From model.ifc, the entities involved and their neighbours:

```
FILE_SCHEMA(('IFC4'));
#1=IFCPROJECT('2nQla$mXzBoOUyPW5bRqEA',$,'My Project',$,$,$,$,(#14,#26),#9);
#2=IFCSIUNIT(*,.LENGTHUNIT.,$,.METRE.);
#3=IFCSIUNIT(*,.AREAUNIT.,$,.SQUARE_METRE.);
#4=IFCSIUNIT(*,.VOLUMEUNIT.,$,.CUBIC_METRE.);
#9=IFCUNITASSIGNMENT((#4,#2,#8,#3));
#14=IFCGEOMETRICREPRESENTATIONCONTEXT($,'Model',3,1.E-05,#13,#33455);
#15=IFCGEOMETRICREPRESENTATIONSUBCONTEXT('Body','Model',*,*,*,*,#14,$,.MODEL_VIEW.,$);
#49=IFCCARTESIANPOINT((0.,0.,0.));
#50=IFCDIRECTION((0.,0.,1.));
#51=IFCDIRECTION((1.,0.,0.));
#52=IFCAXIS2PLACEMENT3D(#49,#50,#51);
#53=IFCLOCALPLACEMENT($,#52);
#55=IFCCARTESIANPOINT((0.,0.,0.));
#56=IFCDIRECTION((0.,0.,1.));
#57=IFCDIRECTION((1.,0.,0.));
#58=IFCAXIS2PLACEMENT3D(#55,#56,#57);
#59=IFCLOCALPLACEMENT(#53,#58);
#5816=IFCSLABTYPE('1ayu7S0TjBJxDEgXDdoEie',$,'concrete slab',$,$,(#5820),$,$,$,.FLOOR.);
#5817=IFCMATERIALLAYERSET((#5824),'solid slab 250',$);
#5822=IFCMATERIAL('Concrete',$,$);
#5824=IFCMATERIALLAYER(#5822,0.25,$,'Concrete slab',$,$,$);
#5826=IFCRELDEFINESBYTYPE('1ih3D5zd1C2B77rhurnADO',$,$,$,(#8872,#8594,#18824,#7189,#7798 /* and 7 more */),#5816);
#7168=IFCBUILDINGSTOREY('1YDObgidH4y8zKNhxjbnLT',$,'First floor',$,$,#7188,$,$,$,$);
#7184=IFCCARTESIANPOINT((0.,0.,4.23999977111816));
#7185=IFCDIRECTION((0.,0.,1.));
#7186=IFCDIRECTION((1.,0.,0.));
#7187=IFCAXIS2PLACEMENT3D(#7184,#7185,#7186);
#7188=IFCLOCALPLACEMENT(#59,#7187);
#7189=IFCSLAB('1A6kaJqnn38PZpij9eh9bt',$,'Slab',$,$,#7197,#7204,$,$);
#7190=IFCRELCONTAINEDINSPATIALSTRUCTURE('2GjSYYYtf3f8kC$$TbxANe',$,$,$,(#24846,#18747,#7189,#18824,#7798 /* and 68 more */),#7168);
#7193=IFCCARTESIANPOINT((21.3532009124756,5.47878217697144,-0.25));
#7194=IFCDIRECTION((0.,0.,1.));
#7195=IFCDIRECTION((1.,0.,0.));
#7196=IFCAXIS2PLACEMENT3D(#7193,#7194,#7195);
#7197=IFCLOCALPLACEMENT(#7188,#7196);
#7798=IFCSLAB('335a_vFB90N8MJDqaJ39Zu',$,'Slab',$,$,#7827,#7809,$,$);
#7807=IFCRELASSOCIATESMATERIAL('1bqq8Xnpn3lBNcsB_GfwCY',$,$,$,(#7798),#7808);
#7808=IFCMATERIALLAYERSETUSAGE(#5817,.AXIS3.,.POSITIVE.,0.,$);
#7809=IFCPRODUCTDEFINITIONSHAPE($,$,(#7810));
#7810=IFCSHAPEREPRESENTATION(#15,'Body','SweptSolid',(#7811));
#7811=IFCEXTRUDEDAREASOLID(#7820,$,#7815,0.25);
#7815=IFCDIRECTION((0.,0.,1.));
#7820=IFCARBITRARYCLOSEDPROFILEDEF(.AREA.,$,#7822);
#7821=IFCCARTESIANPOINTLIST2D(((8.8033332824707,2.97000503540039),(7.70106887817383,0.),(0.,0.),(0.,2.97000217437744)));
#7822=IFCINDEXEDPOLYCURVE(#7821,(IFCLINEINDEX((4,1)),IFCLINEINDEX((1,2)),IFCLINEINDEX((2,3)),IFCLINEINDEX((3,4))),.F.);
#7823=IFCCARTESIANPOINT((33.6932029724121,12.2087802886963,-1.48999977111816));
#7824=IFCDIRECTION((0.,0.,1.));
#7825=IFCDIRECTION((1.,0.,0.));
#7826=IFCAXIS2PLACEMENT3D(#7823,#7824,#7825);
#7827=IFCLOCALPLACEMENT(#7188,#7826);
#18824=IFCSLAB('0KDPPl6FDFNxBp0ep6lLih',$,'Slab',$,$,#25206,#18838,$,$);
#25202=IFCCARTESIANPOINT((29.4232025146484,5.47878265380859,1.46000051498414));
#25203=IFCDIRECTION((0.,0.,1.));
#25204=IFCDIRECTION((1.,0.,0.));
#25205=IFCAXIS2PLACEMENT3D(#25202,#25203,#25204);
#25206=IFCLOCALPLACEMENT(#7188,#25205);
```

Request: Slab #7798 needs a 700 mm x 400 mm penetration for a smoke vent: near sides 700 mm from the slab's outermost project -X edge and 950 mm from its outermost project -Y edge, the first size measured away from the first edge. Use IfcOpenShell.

```python
import numpy as np
import ifcopenshell
import ifcopenshell.api.feature
import ifcopenshell.api.geometry
import ifcopenshell.api.root
import ifcopenshell.geom
import ifcopenshell.util.placement
import ifcopenshell.util.representation
import ifcopenshell.util.shape
import ifcopenshell.util.unit

model = ifcopenshell.open("model.ifc")
unit_scale = ifcopenshell.util.unit.calculate_unit_scale(model)
settings = ifcopenshell.geom.settings()


def volume(element):
    """Net volume in cubic metres, openings subtracted."""
    shape = ifcopenshell.geom.create_shape(settings, element)
    return ifcopenshell.util.shape.get_volume(shape.geometry)


slab = model.by_guid("335a_vFB90N8MJDqaJ39Zu")
before = volume(slab)

# Extent in the slab's own axes, in metres. The edges named are its -X and -Y sides.
slab_shape = ifcopenshell.geom.create_shape(settings, slab)
vertices = ifcopenshell.util.shape.get_vertices(slab_shape.geometry)
x_min, y_min, bottom = vertices.min(axis=0)
top = vertices[:, 2].max()

opening = ifcopenshell.api.root.create_entity(model, ifc_class="IfcOpeningElement", name="Smoke vent opening", predefined_type="OPENING")
context = ifcopenshell.util.representation.get_context(model, "Model", "Body", "MODEL_VIEW")
width, depth = 0.7, 0.4
outline = [(0.0, 0.0), (width, 0.0), (width, depth), (0.0, depth), (0.0, 0.0)]
# Overshoot both faces by 50 mm so the cut is clean.
shape = ifcopenshell.api.geometry.add_slab_representation(
    model, context=context, depth=top - bottom + 0.1, polyline=outline
)
ifcopenshell.api.geometry.assign_representation(model, product=opening, representation=shape)

matrix = ifcopenshell.util.placement.get_local_placement(slab.ObjectPlacement)
matrix[:, 3] = matrix @ np.append(np.array([x_min + 0.7, y_min + 0.95, bottom - 0.05]) / unit_scale, 1.0)
ifcopenshell.api.geometry.edit_object_placement(model, product=opening, matrix=matrix, is_si=False)
ifcopenshell.api.feature.add_feature(model, feature=opening, element=slab)

after = volume(slab)

print(f"slab volume {before:.3f} -> {after:.3f} m3")

model.write("model_v2.ifc")
```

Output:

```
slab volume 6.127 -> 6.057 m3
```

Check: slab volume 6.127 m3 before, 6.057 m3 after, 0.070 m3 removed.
